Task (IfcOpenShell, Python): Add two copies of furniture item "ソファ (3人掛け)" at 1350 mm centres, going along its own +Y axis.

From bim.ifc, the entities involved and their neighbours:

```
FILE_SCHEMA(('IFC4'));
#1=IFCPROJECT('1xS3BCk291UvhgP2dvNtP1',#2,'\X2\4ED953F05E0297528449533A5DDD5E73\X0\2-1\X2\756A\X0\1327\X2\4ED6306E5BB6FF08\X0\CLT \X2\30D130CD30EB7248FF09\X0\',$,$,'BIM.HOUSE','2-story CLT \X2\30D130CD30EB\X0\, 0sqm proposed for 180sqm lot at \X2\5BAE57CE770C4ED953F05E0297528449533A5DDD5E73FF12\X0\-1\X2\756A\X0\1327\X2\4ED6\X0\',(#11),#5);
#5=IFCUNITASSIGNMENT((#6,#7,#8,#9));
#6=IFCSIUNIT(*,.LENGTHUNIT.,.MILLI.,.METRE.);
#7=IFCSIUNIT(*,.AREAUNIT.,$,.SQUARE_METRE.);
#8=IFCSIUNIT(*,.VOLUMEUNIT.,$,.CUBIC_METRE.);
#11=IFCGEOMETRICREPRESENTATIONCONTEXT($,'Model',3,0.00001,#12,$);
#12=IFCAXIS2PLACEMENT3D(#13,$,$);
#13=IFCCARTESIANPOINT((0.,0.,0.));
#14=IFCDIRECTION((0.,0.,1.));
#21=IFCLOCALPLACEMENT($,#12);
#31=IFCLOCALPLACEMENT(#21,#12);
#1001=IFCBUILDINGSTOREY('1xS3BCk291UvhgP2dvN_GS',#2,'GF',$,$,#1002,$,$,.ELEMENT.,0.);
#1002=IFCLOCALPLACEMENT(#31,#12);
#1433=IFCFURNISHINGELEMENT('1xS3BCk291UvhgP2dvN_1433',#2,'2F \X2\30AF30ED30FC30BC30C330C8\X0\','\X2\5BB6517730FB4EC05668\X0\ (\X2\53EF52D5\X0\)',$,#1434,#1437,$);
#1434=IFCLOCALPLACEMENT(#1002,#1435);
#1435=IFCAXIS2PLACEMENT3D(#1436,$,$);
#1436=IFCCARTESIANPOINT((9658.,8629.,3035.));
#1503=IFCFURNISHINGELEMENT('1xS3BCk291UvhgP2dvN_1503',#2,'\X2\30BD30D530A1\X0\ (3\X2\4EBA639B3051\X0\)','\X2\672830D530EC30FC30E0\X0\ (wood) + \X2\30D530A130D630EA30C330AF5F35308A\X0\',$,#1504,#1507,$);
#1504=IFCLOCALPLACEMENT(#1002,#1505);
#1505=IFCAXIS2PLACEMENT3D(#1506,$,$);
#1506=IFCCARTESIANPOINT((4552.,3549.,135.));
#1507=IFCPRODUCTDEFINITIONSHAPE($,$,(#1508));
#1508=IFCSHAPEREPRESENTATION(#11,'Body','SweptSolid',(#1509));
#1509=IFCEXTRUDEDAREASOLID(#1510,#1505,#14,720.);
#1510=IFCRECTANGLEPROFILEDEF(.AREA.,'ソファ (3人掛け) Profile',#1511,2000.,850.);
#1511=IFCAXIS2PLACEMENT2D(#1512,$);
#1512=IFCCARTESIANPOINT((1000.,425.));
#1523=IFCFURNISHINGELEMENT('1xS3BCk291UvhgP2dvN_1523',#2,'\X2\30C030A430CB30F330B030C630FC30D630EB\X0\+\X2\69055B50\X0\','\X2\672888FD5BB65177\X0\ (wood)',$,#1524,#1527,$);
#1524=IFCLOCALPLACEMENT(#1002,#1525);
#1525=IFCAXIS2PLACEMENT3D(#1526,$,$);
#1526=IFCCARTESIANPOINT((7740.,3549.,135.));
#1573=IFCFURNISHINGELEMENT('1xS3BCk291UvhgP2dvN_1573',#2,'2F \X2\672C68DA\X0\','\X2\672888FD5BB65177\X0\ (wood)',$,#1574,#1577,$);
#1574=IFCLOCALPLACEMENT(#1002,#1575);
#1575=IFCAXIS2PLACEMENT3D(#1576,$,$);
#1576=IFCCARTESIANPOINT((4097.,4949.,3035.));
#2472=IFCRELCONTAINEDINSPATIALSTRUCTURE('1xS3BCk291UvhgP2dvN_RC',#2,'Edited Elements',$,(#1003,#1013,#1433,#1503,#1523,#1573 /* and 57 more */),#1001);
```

```python
import ifcopenshell
import ifcopenshell.api.geometry
import ifcopenshell.api.root
import ifcopenshell.util.element
import ifcopenshell.util.placement

model = ifcopenshell.open("bim.ifc")


def reuse_history(source, copy):
    """copy_class also copies each property set's owner history, people and application; keep the originals."""
    for rel in copy.IsDefinedBy:
        if rel.is_a("IfcRelDefinesByProperties") and (history := rel.RelatingPropertyDefinition.OwnerHistory):
            rel.RelatingPropertyDefinition.OwnerHistory = source.OwnerHistory
            ifcopenshell.util.element.remove_deep2(model, history)


source = model.by_id(1503)
base = ifcopenshell.util.placement.get_local_placement(source.ObjectPlacement)
step = base[:3, 1] * 1350.0

for i in range(1, 3):
    copy = ifcopenshell.api.root.copy_class(model, product=source)
    copy.Representation = ifcopenshell.util.element.copy_deep(
        model, source.Representation, exclude=["IfcGeometricRepresentationContext", "IfcRepresentationMap"]
    )
    reuse_history(source, copy)
    matrix = base.copy()
    matrix[:3, 3] += i * step
    print("added at", matrix[:3, 3].round(3) + 0.0)
    ifcopenshell.api.geometry.edit_object_placement(model, product=copy, matrix=matrix, is_si=False)

model.write("bim_updated.ifc")
```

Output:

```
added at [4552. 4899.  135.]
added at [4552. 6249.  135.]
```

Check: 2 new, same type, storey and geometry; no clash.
